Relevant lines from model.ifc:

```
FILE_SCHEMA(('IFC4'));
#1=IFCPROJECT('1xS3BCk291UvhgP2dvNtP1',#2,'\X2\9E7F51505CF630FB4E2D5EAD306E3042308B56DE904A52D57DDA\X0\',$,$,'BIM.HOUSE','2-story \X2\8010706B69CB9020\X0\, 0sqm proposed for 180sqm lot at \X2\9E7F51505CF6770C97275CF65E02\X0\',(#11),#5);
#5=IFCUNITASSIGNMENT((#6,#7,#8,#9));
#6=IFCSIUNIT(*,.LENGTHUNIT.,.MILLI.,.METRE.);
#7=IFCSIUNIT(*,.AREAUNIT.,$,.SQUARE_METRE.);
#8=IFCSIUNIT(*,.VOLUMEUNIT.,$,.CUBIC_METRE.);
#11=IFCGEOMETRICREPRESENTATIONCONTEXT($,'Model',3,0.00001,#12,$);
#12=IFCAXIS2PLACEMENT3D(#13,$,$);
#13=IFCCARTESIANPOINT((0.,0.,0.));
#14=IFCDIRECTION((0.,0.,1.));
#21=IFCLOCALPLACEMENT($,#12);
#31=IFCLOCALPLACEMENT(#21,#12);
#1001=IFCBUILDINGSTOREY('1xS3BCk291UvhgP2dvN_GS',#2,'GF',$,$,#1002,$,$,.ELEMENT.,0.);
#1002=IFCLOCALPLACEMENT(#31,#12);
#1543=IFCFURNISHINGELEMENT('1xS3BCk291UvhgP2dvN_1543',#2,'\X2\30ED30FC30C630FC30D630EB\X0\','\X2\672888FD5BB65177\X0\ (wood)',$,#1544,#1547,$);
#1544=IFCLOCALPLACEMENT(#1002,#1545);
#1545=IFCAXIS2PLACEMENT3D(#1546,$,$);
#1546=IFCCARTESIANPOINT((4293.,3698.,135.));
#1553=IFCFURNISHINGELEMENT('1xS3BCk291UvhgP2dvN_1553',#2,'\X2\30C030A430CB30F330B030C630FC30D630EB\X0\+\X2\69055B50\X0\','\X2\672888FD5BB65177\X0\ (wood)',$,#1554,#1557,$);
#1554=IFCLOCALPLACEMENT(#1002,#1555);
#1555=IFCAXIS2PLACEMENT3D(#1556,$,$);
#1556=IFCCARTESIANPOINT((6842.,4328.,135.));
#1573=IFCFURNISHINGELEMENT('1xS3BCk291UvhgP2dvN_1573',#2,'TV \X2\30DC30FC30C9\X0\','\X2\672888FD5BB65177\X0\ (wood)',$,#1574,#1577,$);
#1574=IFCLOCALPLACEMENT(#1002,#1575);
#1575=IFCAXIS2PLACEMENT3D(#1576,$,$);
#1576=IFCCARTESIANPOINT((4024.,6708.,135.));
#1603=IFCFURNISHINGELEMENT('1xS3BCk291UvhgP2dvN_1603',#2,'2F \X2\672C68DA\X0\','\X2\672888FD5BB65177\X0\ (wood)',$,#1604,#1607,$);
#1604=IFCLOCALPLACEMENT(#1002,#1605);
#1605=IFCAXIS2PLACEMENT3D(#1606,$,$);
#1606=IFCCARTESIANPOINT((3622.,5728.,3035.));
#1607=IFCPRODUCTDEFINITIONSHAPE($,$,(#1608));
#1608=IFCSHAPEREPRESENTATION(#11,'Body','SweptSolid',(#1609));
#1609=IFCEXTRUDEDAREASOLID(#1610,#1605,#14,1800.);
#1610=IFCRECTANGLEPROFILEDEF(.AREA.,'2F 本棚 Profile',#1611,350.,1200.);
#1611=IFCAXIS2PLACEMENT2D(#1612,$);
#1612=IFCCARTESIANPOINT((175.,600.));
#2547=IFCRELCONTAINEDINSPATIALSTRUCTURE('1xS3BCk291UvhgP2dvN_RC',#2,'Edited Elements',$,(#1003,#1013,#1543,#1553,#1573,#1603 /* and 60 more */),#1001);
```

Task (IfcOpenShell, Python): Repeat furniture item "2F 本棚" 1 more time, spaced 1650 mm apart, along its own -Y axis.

```python
import ifcopenshell
import ifcopenshell.api.geometry
import ifcopenshell.api.root
import ifcopenshell.util.element
import ifcopenshell.util.placement
import ifcopenshell.util.unit

model = ifcopenshell.open("model.ifc")
unit_scale = ifcopenshell.util.unit.calculate_unit_scale(model)


def reuse_history(source, copy):
    """copy_class also copies each property set's owner history, people and application; keep the originals."""
    for rel in copy.IsDefinedBy:
        if rel.is_a("IfcRelDefinesByProperties") and (history := rel.RelatingPropertyDefinition.OwnerHistory):
            rel.RelatingPropertyDefinition.OwnerHistory = source.OwnerHistory
            ifcopenshell.util.element.remove_deep2(model, history)


source = model.by_id(1603)
base = ifcopenshell.util.placement.get_local_placement(source.ObjectPlacement)
step = -base[:3, 1] * 1.65 / unit_scale

for i in range(1, 2):
    copy = ifcopenshell.api.root.copy_class(model, product=source)
    copy.Representation = ifcopenshell.util.element.copy_deep(
        model, source.Representation, exclude=["IfcGeometricRepresentationContext", "IfcRepresentationMap"]
    )
    reuse_history(source, copy)
    matrix = base.copy()
    matrix[:3, 3] += i * step
    print("added at", matrix[:3, 3].round(3) + 0.0)
    ifcopenshell.api.geometry.edit_object_placement(model, product=copy, matrix=matrix, is_si=False)

model.write("model-out.ifc")
```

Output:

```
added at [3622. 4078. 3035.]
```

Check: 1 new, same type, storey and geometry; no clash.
